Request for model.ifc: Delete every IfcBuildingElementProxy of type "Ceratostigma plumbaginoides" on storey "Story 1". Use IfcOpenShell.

First a look at what the model holds.

```python
import ifcopenshell
import ifcopenshell.util.element

model = ifcopenshell.open("model.ifc")
print(model.schema)
storey = next(s for s in model.by_type("IfcBuildingStorey") if s.Name == "Story 1")
proxies = [e for e in ifcopenshell.util.element.get_decomposition(storey) if e.is_a("IfcBuildingElementProxy")]
seen = {}
for e in proxies:
    element_type = ifcopenshell.util.element.get_type(e)
    name = element_type.Name if element_type not in (None, e) else None
    seen[name] = seen.get(name, 0) + 1
for name, count in sorted(seen.items(), key=str):
    print(count, "x", name)
```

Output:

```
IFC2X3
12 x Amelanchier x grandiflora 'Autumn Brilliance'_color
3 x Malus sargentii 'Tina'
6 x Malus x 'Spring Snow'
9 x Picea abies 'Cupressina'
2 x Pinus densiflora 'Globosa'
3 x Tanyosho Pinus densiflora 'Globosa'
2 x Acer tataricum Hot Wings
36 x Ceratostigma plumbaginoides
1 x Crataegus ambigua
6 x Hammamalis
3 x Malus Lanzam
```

```python
import ifcopenshell
import ifcopenshell.api.root
import ifcopenshell.util.element

model = ifcopenshell.open("model.ifc")

storey = next(s for s in model.by_type("IfcBuildingStorey") if s.Name == "Story 1")
proxies = [e for e in ifcopenshell.util.element.get_decomposition(storey) if e.is_a("IfcBuildingElementProxy")]
targets = [e for e in proxies if (t := ifcopenshell.util.element.get_type(e)) not in (None, e) and t.Name == "Ceratostigma plumbaginoides"]

for e in targets:
    ifcopenshell.api.root.remove_product(model, product=e)
print(len(targets), "removed")

model.write("model_edited.ifc")
```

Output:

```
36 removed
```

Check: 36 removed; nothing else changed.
